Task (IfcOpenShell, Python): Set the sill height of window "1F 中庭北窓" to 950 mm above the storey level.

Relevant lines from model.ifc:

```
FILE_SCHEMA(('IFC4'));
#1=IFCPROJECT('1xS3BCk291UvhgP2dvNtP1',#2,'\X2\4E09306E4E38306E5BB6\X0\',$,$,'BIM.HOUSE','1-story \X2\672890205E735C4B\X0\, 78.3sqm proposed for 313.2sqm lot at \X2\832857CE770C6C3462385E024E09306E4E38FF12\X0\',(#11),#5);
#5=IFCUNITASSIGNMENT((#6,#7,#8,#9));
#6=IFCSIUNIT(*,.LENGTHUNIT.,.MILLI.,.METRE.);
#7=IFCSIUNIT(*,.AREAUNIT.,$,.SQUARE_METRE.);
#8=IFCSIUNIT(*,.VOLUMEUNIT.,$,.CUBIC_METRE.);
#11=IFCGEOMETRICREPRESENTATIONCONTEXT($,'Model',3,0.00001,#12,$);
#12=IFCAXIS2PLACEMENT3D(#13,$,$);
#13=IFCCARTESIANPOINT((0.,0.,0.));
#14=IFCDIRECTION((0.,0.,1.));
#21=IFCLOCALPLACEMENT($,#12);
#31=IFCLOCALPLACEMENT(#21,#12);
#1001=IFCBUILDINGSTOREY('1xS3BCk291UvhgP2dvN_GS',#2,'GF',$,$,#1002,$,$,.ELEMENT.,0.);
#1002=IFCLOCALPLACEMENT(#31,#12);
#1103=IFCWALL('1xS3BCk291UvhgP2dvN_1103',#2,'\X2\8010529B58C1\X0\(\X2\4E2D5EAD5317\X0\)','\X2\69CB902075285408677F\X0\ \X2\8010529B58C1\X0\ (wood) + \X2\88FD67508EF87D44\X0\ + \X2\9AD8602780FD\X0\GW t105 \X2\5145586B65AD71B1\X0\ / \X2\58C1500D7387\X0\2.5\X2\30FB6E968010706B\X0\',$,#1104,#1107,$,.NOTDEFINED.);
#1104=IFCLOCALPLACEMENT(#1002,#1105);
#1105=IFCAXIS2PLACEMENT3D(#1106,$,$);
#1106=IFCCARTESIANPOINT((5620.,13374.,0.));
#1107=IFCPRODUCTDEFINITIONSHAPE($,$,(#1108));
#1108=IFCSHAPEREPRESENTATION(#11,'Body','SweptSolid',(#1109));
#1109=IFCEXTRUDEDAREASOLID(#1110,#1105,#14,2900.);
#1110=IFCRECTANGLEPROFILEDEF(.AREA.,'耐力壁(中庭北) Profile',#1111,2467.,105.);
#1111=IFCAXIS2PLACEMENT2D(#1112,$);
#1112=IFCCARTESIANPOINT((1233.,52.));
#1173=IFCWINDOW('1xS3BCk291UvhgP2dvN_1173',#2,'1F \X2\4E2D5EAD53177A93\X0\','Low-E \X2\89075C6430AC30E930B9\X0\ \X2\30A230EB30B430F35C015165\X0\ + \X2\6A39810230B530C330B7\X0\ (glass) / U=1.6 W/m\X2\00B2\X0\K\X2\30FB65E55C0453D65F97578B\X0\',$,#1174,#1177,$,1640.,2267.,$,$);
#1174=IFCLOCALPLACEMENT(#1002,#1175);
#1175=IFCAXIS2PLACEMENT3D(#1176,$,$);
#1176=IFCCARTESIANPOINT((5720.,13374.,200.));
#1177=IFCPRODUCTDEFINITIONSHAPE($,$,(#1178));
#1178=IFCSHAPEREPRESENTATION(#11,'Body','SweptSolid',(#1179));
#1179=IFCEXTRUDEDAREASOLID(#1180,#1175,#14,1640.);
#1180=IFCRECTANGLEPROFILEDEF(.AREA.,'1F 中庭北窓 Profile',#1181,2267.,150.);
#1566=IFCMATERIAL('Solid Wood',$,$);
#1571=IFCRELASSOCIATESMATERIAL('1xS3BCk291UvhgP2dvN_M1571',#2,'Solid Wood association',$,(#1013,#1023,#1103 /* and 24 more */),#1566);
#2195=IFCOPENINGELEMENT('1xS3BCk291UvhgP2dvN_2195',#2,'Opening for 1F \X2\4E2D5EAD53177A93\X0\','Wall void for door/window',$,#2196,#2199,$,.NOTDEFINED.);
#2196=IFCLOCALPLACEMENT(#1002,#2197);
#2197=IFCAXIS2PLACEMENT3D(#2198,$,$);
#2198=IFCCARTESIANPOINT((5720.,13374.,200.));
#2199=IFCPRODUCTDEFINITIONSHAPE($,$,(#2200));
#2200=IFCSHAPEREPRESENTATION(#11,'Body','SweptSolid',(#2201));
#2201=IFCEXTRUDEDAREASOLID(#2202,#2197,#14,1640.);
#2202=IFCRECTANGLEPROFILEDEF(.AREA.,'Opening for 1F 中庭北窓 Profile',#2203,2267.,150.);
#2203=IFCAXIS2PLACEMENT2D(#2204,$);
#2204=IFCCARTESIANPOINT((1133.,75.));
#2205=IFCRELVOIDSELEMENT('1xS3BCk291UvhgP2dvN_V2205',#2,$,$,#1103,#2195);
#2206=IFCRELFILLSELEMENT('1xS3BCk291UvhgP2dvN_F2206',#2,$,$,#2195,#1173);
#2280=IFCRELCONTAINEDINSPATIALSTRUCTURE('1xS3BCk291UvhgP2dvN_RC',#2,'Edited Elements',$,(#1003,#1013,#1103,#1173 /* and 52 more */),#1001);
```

```python
import numpy as np
import ifcopenshell
import ifcopenshell.api.geometry
import ifcopenshell.geom
import ifcopenshell.util.element
import ifcopenshell.util.placement
import ifcopenshell.util.shape
import ifcopenshell.util.unit

model = ifcopenshell.open("model.ifc")
unit_scale = ifcopenshell.util.unit.calculate_unit_scale(model)

window = model.by_guid("1xS3BCk291UvhgP2dvN_1173")
opening = window.FillsVoids[0].RelatingOpeningElement
storey = ifcopenshell.util.element.get_container(window, ifc_class="IfcBuildingStorey")
level = ifcopenshell.util.placement.get_local_placement(storey.ObjectPlacement)[2, 3]

# The opening's origin need not be at the sill, so measure its lowest point.
shape = ifcopenshell.geom.create_shape(ifcopenshell.geom.settings(), opening)
bottom = ifcopenshell.util.shape.get_shape_bottom_elevation(shape, shape.geometry) / unit_scale
dz = level + 0.95 / unit_scale - bottom

shift = np.array([0.0, 0.0, dz])
# The window is not placed relative to its opening, so move both.
for product in (opening, window):
    matrix = ifcopenshell.util.placement.get_local_placement(product.ObjectPlacement)
    matrix[:3, 3] += shift
    ifcopenshell.api.geometry.edit_object_placement(model, product=product, matrix=matrix, is_si=False)

print(f"moved by {dz * unit_scale:+.3f} m")

model.write("model_v2.ifc")
```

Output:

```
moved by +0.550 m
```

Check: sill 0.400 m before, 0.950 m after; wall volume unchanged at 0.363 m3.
